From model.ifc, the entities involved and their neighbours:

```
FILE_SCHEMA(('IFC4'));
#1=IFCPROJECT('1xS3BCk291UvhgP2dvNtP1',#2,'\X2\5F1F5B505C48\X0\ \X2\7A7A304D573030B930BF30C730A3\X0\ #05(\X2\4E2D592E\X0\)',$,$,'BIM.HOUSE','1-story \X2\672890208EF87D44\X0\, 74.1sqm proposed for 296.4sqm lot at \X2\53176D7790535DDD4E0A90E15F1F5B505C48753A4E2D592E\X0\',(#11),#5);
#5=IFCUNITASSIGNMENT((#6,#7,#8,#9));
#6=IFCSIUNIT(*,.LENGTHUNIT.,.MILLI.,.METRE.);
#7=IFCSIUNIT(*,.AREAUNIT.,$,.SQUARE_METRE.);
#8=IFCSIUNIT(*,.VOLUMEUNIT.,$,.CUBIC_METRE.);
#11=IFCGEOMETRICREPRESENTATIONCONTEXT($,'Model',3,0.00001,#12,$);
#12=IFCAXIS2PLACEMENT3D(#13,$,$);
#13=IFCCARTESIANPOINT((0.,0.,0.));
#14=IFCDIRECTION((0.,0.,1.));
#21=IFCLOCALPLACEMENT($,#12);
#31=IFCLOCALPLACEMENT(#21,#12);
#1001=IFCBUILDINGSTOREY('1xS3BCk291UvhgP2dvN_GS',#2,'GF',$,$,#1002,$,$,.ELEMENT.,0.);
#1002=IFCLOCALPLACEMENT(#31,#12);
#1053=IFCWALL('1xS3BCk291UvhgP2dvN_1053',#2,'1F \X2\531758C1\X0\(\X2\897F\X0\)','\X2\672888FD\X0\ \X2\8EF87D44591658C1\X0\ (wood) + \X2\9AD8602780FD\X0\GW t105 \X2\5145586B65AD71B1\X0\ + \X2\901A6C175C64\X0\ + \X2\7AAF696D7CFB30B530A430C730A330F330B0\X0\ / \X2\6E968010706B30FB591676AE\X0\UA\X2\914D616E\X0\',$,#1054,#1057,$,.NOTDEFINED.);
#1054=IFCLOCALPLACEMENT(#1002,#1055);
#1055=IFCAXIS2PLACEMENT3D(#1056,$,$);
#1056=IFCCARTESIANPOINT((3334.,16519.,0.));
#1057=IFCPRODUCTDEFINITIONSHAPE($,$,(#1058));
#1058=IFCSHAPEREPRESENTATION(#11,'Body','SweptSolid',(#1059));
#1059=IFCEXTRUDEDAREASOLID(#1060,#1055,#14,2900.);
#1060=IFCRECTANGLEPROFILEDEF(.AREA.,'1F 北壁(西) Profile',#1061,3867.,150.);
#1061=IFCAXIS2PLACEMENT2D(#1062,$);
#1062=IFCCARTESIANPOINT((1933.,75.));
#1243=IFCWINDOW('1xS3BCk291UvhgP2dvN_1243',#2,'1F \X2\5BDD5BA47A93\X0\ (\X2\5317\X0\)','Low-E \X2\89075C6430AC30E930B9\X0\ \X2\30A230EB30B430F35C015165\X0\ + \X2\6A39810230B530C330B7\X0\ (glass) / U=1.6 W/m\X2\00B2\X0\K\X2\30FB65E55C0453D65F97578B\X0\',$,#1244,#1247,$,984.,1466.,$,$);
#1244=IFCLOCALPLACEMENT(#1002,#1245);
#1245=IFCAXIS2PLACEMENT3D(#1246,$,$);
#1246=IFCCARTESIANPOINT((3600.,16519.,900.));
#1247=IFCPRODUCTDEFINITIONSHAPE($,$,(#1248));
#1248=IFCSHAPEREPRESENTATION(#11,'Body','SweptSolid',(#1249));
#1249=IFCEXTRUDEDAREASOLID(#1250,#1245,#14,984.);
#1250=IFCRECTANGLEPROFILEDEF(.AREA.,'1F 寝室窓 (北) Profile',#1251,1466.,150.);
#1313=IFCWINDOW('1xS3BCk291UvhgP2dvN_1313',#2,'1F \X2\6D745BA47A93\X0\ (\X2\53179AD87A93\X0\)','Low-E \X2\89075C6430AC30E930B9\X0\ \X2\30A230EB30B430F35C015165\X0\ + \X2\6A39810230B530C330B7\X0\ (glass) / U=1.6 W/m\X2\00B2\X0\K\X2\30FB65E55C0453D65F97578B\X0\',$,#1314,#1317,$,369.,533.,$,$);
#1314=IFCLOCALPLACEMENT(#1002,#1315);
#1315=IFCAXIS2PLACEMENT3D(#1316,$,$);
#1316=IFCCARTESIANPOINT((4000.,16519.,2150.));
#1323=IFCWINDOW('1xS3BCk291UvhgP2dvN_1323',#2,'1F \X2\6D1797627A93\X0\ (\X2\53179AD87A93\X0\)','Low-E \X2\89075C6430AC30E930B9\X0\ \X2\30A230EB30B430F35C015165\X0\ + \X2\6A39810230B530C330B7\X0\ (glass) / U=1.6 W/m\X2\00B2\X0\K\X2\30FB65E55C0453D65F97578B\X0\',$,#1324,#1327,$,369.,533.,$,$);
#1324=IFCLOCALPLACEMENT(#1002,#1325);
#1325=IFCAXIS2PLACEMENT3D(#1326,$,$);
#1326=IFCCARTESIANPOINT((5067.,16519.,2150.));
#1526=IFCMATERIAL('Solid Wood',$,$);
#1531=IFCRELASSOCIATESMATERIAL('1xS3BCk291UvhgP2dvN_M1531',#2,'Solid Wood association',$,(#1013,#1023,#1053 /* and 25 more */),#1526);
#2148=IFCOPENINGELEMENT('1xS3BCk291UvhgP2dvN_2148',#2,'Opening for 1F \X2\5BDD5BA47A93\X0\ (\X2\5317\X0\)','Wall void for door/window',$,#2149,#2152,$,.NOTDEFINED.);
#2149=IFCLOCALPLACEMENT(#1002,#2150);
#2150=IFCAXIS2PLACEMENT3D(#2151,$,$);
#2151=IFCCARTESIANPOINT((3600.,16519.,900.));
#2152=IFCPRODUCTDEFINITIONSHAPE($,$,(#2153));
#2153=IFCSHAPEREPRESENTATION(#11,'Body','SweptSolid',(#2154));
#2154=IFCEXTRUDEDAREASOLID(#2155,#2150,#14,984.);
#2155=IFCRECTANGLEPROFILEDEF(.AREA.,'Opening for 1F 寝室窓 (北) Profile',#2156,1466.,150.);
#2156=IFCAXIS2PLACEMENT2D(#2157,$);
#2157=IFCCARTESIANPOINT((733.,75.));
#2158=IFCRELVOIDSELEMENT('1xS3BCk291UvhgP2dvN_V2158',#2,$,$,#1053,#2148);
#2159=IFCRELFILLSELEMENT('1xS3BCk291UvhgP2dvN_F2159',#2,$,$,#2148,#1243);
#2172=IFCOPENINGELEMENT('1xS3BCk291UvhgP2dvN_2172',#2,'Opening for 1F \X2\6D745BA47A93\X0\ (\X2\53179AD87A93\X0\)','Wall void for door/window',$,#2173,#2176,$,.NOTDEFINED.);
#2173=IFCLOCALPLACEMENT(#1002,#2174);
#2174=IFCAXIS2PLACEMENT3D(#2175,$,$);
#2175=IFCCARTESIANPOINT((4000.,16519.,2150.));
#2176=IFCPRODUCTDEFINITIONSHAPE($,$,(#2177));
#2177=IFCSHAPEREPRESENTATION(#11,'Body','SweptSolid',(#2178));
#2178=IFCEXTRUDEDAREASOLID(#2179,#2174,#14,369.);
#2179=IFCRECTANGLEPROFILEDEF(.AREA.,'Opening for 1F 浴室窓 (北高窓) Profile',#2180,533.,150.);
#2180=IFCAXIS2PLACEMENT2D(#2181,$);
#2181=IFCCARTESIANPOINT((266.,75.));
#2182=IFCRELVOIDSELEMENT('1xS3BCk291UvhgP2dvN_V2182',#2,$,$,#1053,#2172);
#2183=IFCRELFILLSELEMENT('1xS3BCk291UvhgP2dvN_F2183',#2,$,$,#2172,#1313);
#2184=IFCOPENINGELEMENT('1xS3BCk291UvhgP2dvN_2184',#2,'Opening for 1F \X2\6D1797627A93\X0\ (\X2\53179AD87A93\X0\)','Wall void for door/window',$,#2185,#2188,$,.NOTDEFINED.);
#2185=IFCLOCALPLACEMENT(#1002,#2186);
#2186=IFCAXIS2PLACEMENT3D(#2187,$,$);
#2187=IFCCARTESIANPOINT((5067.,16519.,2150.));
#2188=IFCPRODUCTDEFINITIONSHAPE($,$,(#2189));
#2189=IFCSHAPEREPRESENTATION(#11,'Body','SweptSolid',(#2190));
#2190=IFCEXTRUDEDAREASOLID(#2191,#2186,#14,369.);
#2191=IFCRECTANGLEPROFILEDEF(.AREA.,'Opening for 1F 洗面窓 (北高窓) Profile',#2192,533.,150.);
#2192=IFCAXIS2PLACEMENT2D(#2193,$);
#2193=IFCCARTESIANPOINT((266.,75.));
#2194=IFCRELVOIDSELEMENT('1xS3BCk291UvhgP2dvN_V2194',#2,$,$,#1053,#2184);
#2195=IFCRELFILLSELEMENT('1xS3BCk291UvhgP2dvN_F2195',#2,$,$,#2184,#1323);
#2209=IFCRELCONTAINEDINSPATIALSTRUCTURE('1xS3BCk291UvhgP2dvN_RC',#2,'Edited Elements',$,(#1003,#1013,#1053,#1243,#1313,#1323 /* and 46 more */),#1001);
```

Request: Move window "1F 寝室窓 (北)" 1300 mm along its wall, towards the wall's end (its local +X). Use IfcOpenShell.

```python
import ifcopenshell
import ifcopenshell.api.geometry
import ifcopenshell.util.placement

model = ifcopenshell.open("model.ifc")

window = model.by_guid("1xS3BCk291UvhgP2dvN_1243")
opening = window.FillsVoids[0].RelatingOpeningElement
wall = opening.VoidsElements[0].RelatingBuildingElement

wall_matrix = ifcopenshell.util.placement.get_local_placement(wall.ObjectPlacement)
shift = wall_matrix[:3, 0] * 1300.0
before = ifcopenshell.util.placement.get_local_placement(window.ObjectPlacement)[:3, 3].copy()

# The window is not placed relative to its opening, so move both.
for product in (opening, window):
    matrix = ifcopenshell.util.placement.get_local_placement(product.ObjectPlacement)
    matrix[:3, 3] += shift
    ifcopenshell.api.geometry.edit_object_placement(model, product=product, matrix=matrix, is_si=False)

after = ifcopenshell.util.placement.get_local_placement(window.ObjectPlacement)[:3, 3]
print("window moved by", (after - before).round(3) + 0.0)

model.write("model_v2.ifc")
```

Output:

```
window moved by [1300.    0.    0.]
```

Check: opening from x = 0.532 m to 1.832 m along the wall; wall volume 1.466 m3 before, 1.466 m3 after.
